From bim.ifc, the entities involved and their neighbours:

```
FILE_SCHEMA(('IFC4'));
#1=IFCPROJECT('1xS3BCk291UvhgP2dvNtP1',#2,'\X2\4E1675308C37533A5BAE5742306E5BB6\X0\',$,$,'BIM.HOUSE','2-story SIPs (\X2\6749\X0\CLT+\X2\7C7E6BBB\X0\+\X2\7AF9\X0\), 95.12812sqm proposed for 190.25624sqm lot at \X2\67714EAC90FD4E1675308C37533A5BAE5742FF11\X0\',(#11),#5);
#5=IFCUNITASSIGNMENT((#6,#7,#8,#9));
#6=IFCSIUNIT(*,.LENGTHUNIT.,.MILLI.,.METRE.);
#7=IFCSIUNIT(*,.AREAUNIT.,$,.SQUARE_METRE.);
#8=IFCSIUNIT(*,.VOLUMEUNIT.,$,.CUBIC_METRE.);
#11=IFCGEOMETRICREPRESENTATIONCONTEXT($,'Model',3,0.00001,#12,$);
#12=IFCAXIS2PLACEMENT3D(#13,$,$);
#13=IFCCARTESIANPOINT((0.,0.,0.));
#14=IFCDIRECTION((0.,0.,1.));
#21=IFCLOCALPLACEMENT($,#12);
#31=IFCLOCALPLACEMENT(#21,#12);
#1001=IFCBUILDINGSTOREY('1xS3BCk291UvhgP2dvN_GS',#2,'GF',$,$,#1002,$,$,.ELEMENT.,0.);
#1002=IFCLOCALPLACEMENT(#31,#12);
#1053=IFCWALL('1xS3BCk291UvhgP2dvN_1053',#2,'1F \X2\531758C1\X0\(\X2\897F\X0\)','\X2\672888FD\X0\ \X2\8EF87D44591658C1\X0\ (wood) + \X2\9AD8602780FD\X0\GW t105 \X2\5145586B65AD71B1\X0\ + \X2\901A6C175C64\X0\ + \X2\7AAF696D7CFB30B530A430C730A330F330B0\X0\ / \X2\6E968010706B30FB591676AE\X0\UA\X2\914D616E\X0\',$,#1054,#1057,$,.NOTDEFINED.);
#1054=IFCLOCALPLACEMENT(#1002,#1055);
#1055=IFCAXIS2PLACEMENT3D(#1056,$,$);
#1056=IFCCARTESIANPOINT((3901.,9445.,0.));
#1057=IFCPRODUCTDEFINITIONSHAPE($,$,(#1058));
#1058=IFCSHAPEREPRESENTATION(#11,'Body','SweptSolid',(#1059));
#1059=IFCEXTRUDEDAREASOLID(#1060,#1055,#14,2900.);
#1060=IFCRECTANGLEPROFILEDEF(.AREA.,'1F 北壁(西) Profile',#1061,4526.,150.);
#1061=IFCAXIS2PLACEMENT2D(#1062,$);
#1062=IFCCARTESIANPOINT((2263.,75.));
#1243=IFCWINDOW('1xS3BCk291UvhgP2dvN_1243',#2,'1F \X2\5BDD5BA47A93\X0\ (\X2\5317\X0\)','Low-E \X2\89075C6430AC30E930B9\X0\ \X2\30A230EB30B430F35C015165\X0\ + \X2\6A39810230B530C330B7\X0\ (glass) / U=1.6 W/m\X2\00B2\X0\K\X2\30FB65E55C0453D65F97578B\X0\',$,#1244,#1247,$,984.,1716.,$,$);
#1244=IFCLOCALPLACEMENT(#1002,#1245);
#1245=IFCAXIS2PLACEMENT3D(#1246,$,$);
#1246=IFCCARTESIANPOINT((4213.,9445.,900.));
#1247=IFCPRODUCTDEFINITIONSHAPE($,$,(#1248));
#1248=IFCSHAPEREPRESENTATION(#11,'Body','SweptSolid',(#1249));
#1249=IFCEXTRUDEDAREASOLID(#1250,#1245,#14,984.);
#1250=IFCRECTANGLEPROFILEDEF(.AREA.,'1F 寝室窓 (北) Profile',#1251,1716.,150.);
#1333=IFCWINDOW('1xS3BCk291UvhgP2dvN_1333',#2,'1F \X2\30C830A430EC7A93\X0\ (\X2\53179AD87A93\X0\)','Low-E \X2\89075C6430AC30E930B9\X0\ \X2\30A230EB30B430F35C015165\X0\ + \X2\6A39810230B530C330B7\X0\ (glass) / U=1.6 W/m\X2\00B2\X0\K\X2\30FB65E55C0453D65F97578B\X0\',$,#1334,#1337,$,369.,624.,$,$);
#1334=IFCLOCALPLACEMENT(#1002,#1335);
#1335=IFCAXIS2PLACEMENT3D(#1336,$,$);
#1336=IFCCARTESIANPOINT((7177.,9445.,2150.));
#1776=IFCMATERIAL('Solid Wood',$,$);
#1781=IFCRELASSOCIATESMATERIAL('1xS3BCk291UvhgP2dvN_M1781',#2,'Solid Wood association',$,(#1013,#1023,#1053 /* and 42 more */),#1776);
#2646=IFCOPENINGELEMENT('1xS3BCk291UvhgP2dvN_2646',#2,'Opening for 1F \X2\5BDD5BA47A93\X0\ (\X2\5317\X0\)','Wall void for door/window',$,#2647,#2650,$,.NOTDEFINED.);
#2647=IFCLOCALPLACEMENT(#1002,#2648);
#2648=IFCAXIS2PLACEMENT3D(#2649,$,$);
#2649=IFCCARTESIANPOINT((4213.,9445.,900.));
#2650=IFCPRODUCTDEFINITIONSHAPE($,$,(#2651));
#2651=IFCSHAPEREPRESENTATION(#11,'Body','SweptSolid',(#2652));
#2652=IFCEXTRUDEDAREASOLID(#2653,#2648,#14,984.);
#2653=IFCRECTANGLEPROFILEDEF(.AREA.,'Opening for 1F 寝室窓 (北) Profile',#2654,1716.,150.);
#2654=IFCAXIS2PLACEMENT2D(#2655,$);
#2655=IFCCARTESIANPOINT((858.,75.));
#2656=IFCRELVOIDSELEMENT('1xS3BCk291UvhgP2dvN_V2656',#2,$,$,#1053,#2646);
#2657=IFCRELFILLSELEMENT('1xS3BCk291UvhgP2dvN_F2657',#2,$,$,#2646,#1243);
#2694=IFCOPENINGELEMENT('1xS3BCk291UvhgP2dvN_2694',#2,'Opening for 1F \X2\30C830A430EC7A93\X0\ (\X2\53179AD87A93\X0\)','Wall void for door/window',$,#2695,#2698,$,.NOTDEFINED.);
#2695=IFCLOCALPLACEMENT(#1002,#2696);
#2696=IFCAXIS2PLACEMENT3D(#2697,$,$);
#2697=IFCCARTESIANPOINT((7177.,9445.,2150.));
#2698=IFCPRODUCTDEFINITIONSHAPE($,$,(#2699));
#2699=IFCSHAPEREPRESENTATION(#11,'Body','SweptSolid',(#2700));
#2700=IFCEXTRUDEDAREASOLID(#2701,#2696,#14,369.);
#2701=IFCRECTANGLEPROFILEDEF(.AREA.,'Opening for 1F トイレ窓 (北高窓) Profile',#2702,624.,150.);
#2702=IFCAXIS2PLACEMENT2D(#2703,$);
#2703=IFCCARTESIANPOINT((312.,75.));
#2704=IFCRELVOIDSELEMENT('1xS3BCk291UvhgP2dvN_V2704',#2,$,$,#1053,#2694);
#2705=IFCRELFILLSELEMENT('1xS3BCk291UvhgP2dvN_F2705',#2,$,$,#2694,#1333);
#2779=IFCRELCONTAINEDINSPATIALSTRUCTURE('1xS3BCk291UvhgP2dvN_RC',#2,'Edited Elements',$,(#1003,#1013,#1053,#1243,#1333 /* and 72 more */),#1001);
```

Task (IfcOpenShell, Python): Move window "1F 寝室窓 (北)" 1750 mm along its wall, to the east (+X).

```python
import ifcopenshell
import ifcopenshell.api.geometry
import ifcopenshell.util.placement
import ifcopenshell.util.unit

model = ifcopenshell.open("bim.ifc")
unit_scale = ifcopenshell.util.unit.calculate_unit_scale(model)

window = model.by_guid("1xS3BCk291UvhgP2dvN_1243")
opening = window.FillsVoids[0].RelatingOpeningElement
wall = opening.VoidsElements[0].RelatingBuildingElement

wall_matrix = ifcopenshell.util.placement.get_local_placement(wall.ObjectPlacement)
shift = wall_matrix[:3, 0] * 1.75 / unit_scale
before = ifcopenshell.util.placement.get_local_placement(window.ObjectPlacement)[:3, 3].copy()

# The window is not placed relative to its opening, so move both.
for product in (opening, window):
    matrix = ifcopenshell.util.placement.get_local_placement(product.ObjectPlacement)
    matrix[:3, 3] += shift
    ifcopenshell.api.geometry.edit_object_placement(model, product=product, matrix=matrix, is_si=False)

after = ifcopenshell.util.placement.get_local_placement(window.ObjectPlacement)[:3, 3]
print("window moved by", (after - before).round(3) + 0.0)

model.write("bim_rev.ifc")
```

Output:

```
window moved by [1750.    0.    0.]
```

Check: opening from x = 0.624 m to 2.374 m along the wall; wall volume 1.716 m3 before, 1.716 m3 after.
